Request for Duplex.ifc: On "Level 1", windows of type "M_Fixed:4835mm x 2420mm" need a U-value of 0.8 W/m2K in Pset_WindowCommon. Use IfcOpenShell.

First a look at what the model holds.

```python
import ifcopenshell
import ifcopenshell.util.element

model = ifcopenshell.open("Duplex.ifc")
print(model.schema)
storey = next(s for s in model.by_type("IfcBuildingStorey") if s.Name == "Level 1")
windows = [e for e in ifcopenshell.util.element.get_decomposition(storey) if e.is_a("IfcWindow")]
seen = {}
for e in windows:
    element_type = ifcopenshell.util.element.get_type(e)
    key = (element_type.Name if element_type != e and element_type else None, ifcopenshell.util.element.get_pset(e, "Pset_WindowCommon", "ThermalTransmittance"))
    seen[key] = seen.get(key, 0) + 1
for (name, value), count in sorted(seen.items(), key=str):
    print(count, "x", name, "|", value)
```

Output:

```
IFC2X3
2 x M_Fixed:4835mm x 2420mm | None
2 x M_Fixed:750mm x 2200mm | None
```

```python
import ifcopenshell
import ifcopenshell.api.pset
import ifcopenshell.util.element

model = ifcopenshell.open("Duplex.ifc")

storey = next(s for s in model.by_type("IfcBuildingStorey") if s.Name == "Level 1")
windows = [e for e in ifcopenshell.util.element.get_decomposition(storey) if e.is_a("IfcWindow")]

count = 0
for e in windows:
    element_type = ifcopenshell.util.element.get_type(e)
    if element_type in (None, e) or element_type.Name != "M_Fixed:4835mm x 2420mm":
        continue
    # add_pset returns the element's existing set when there is one.
    pset = ifcopenshell.api.pset.add_pset(model, product=e, name="Pset_WindowCommon")
    ifcopenshell.api.pset.edit_pset(model, pset=pset, properties={"ThermalTransmittance": 0.8})
    count += 1

print(count, "windows updated")

model.write("Duplex_rev.ifc")
```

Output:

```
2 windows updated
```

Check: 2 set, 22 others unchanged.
